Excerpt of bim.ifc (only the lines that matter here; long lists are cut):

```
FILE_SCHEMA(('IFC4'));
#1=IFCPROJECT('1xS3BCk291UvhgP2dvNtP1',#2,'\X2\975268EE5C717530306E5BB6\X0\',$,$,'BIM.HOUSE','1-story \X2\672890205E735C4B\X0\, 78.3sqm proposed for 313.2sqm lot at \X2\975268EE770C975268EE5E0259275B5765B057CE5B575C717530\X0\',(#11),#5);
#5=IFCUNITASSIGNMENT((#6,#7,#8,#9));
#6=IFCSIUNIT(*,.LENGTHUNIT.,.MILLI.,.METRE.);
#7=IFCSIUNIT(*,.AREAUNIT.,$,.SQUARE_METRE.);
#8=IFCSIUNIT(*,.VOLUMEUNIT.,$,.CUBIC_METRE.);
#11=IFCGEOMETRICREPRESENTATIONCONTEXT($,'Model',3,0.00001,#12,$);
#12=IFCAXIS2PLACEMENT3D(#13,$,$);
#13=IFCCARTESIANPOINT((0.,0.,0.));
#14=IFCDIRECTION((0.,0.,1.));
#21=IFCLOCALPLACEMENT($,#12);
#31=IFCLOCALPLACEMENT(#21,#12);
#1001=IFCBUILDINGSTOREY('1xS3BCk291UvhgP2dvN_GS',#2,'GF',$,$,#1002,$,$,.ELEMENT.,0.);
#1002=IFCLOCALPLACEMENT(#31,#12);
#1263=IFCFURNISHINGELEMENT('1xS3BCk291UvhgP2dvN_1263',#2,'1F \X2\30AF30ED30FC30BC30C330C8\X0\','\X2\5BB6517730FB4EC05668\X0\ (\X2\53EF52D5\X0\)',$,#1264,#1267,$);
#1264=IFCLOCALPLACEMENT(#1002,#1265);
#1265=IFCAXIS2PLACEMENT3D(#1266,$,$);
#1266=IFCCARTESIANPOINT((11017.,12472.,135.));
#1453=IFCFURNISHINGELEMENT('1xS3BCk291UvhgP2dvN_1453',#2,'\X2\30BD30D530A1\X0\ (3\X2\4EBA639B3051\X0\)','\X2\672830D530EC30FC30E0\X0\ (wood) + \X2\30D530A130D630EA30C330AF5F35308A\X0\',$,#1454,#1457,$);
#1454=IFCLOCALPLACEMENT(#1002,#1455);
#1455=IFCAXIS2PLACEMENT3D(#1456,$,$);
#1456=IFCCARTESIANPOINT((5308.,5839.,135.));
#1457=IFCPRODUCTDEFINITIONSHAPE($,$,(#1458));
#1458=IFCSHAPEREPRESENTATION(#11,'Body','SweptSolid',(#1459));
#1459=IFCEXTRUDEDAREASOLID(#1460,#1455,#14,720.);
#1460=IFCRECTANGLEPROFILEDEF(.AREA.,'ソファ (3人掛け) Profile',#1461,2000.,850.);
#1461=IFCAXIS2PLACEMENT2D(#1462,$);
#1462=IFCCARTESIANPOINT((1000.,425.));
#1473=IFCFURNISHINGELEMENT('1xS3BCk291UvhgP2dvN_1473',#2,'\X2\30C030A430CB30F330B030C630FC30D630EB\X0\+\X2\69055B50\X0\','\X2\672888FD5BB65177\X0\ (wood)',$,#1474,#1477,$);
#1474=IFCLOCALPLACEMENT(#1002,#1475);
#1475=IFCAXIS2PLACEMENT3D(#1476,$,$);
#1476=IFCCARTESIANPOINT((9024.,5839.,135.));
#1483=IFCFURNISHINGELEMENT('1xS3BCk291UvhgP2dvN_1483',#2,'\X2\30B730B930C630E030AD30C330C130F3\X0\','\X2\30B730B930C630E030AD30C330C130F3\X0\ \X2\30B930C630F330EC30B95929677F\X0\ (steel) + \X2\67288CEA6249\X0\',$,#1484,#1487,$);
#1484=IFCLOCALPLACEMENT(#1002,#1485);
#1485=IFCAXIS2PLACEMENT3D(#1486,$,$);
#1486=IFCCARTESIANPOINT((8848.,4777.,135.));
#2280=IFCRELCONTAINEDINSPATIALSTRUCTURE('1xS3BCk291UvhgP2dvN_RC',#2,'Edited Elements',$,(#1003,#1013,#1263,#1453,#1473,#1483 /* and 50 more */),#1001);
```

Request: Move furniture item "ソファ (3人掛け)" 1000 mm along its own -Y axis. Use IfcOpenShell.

```python
import ifcopenshell
import ifcopenshell.api.geometry
import ifcopenshell.util.placement
import ifcopenshell.util.unit

model = ifcopenshell.open("bim.ifc")
unit_scale = ifcopenshell.util.unit.calculate_unit_scale(model)

item = model.by_guid("1xS3BCk291UvhgP2dvN_1453")
matrix = ifcopenshell.util.placement.get_local_placement(item.ObjectPlacement)
matrix[:3, 3] -= matrix[:3, 1] * 1 / unit_scale
ifcopenshell.api.geometry.edit_object_placement(model, product=item, matrix=matrix, is_si=False)

print(ifcopenshell.util.placement.get_local_placement(item.ObjectPlacement).round(3) + 0.0)

model.write("bim_v2.ifc")
```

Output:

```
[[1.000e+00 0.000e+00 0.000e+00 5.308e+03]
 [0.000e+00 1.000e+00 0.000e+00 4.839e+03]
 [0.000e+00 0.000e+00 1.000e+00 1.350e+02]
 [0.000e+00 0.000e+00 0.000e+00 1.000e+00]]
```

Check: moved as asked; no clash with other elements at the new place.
